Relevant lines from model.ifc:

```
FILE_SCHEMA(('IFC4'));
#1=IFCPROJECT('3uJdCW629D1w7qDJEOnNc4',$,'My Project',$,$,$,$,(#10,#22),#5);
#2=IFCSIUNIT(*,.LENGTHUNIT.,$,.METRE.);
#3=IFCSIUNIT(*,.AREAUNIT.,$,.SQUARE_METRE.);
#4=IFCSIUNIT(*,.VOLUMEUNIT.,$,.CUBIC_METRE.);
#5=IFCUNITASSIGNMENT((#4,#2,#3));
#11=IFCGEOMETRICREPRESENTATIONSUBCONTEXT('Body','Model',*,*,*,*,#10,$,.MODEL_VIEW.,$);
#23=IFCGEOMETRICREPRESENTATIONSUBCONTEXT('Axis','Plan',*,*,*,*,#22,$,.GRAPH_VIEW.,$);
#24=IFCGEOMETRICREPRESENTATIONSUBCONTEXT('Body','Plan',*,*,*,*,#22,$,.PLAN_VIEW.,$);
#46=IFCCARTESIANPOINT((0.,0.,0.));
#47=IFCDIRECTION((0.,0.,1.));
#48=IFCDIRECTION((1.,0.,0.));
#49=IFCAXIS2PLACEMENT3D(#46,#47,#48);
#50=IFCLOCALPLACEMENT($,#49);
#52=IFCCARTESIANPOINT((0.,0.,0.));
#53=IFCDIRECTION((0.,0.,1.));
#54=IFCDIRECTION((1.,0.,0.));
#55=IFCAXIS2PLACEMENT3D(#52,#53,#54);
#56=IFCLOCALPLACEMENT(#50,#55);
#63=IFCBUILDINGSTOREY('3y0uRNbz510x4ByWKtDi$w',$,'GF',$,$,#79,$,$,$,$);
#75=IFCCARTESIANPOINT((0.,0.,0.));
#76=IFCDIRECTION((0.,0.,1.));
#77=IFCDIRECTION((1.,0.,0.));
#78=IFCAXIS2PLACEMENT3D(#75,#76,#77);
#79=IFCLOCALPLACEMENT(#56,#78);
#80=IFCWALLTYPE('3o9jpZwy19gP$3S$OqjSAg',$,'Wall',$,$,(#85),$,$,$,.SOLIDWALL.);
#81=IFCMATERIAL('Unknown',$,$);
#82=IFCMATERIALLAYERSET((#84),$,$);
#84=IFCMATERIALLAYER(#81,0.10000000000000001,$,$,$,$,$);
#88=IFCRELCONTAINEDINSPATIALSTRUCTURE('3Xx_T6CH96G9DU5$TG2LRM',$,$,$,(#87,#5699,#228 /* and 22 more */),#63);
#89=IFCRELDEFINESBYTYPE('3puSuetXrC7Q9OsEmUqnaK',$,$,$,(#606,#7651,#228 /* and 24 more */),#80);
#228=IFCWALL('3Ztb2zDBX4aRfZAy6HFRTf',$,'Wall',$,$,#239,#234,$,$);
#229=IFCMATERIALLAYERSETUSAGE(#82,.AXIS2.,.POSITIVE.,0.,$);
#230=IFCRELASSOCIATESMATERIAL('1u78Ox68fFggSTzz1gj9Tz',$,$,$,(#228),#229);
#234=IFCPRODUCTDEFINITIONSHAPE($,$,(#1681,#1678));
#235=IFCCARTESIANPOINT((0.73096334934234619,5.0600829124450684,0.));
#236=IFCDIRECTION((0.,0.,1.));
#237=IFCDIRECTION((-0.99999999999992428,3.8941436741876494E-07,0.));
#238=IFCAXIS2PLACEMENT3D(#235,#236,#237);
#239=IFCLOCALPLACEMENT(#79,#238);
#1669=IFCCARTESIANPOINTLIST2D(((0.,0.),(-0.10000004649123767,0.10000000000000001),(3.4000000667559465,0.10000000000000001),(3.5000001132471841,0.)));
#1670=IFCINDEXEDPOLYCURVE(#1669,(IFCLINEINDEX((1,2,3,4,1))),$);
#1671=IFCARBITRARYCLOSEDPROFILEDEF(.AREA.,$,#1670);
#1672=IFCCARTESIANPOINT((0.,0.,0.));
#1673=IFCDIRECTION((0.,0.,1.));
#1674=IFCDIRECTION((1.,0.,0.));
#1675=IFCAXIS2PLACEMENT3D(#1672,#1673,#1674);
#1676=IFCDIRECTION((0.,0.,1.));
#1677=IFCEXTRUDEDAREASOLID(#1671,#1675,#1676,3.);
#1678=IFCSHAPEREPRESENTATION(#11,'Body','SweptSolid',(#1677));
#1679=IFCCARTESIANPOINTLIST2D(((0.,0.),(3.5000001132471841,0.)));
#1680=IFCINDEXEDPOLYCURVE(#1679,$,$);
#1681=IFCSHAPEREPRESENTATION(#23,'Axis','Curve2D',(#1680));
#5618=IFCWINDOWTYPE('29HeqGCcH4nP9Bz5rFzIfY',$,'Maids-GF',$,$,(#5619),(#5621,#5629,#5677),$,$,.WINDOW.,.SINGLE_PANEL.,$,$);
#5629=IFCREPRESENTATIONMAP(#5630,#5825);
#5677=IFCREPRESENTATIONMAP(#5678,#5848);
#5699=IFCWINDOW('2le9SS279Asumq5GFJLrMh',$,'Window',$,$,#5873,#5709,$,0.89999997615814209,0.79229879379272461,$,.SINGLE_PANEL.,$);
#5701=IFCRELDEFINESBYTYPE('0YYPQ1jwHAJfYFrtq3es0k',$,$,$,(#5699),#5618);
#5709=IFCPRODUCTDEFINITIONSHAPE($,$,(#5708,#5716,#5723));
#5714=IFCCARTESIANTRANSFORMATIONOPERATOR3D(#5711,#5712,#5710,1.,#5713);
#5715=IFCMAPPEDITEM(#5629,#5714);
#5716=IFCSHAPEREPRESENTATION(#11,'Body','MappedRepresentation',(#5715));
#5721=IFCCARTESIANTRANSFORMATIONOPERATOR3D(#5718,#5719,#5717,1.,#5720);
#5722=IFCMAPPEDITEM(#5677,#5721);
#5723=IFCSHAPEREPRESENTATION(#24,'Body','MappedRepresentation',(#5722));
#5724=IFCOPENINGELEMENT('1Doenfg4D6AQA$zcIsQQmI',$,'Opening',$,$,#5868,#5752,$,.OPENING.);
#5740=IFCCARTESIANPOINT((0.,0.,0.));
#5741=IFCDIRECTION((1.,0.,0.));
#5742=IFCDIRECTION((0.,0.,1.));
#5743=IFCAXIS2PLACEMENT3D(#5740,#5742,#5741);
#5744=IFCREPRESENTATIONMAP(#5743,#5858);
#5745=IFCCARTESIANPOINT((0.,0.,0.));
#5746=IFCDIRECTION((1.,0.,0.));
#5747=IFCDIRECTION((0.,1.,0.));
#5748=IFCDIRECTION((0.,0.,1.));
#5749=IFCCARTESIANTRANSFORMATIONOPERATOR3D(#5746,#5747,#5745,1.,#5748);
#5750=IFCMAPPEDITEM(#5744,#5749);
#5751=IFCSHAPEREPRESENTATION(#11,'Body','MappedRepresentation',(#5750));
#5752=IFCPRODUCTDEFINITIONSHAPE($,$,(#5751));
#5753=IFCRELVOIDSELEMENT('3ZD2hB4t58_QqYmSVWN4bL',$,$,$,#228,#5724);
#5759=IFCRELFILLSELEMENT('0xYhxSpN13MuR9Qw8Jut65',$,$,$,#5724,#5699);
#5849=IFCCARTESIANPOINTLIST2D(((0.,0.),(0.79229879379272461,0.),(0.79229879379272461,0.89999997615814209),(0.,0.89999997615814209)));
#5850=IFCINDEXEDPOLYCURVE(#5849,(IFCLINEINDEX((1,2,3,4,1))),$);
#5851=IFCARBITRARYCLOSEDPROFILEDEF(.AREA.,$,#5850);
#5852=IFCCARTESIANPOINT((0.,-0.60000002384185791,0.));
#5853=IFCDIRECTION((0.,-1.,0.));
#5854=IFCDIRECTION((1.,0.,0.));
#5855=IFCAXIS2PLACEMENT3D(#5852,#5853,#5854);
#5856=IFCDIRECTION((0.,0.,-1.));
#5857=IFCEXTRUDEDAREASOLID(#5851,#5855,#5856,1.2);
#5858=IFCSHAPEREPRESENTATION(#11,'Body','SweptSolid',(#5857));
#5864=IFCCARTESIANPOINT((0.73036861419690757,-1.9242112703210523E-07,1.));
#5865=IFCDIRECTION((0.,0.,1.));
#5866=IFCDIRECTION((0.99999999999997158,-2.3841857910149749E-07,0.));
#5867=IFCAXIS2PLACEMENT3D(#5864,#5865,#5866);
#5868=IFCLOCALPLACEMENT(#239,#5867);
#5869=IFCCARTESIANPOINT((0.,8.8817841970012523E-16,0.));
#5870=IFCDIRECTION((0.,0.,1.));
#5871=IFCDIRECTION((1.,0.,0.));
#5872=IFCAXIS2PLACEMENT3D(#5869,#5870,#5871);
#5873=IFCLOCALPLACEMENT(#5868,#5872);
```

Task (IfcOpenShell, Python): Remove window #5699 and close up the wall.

```python
import ifcopenshell
import ifcopenshell.api.feature
import ifcopenshell.api.root
import ifcopenshell.geom
import ifcopenshell.util.shape

model = ifcopenshell.open("model.ifc")
settings = ifcopenshell.geom.settings()


def volume(element):
    """Net volume in cubic metres, openings subtracted."""
    shape = ifcopenshell.geom.create_shape(settings, element)
    return ifcopenshell.util.shape.get_volume(shape.geometry)


window = model.by_guid("2le9SS279Asumq5GFJLrMh")
opening = window.FillsVoids[0].RelatingOpeningElement
wall = opening.VoidsElements[0].RelatingBuildingElement
before = volume(wall)

ifcopenshell.api.root.remove_product(model, product=window)
ifcopenshell.api.feature.remove_feature(model, feature=opening)

after = volume(wall)

print(f"wall volume {before:.3f} -> {after:.3f} m3")

model.write("model_edited.ifc")
```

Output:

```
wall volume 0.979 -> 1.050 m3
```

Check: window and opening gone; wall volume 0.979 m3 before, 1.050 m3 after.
